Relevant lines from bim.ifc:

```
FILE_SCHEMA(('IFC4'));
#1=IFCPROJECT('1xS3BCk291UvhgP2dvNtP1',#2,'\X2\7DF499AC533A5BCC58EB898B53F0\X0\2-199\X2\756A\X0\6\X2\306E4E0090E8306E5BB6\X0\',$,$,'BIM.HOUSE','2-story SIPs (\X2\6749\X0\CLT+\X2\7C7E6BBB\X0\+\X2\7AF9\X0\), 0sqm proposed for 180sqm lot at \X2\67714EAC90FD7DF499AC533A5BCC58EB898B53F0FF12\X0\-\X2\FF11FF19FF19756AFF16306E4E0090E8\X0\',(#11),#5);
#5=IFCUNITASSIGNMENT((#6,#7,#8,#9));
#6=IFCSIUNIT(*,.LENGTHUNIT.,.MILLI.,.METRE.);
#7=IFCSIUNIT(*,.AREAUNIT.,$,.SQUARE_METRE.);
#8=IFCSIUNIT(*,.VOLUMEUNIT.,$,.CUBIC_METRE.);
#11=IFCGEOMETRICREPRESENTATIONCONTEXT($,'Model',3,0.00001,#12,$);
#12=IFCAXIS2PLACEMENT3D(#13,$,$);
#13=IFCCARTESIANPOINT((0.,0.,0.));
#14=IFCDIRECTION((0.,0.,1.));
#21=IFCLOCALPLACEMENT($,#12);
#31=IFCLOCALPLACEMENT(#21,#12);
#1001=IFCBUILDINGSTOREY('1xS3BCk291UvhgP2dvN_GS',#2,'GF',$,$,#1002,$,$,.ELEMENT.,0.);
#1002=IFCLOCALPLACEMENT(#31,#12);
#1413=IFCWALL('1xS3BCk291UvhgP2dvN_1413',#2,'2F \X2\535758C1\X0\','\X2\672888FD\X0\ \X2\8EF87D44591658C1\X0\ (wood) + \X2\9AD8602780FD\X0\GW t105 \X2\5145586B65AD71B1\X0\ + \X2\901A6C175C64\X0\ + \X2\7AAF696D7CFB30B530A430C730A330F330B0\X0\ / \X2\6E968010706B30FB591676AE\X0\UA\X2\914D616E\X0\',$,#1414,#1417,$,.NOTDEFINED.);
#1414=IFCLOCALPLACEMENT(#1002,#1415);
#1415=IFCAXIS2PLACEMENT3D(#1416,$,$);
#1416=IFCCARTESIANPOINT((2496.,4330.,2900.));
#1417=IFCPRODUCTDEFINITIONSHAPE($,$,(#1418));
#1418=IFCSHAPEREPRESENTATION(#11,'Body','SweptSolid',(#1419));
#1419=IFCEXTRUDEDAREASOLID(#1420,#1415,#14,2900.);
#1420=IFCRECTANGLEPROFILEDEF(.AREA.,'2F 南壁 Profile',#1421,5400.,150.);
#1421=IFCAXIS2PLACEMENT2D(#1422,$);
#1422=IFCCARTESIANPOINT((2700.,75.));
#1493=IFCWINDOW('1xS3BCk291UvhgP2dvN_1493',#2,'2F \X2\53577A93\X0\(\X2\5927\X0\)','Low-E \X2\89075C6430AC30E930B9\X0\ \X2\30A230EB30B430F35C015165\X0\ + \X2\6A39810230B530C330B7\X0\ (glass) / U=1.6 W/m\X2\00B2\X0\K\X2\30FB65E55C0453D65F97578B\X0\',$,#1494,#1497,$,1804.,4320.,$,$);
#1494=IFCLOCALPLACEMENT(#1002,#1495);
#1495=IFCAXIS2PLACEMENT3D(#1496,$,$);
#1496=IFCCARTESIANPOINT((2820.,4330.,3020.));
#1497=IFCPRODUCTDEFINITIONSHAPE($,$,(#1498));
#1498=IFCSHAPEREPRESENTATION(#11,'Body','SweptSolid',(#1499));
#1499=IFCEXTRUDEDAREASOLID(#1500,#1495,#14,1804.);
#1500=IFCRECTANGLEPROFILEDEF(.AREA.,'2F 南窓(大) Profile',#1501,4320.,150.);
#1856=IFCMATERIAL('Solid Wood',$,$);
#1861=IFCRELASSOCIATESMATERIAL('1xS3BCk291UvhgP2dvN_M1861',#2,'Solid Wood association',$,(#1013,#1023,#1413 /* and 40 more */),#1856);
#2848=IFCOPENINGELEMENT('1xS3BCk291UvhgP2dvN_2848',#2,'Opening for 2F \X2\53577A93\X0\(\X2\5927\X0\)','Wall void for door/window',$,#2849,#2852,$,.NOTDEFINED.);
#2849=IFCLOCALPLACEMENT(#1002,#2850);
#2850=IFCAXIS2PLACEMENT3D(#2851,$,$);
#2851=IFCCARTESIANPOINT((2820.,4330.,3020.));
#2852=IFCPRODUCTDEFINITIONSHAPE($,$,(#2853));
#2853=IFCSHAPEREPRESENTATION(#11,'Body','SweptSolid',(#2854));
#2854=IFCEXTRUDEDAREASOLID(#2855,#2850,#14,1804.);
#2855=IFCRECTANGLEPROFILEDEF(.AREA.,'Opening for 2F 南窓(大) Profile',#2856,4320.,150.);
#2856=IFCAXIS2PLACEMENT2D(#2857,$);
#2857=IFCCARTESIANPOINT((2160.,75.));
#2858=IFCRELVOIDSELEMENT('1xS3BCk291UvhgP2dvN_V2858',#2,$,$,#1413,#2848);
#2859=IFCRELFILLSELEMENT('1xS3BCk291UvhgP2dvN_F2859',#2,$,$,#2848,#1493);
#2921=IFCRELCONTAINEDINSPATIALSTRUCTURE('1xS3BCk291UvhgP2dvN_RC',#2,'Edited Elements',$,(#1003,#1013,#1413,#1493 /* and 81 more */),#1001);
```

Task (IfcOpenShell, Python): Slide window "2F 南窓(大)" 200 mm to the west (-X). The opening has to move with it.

```python
import ifcopenshell
import ifcopenshell.api.geometry
import ifcopenshell.util.placement

model = ifcopenshell.open("bim.ifc")

window = model.by_guid("1xS3BCk291UvhgP2dvN_1493")
opening = window.FillsVoids[0].RelatingOpeningElement
wall = opening.VoidsElements[0].RelatingBuildingElement

wall_matrix = ifcopenshell.util.placement.get_local_placement(wall.ObjectPlacement)
shift = wall_matrix[:3, 0] * -200.0
before = ifcopenshell.util.placement.get_local_placement(window.ObjectPlacement)[:3, 3].copy()

# The window is not placed relative to its opening, so move both.
for product in (opening, window):
    matrix = ifcopenshell.util.placement.get_local_placement(product.ObjectPlacement)
    matrix[:3, 3] += shift
    ifcopenshell.api.geometry.edit_object_placement(model, product=product, matrix=matrix, is_si=False)

after = ifcopenshell.util.placement.get_local_placement(window.ObjectPlacement)[:3, 3]
print("window moved by", (after - before).round(3) + 0.0)

model.write("bim_rev.ifc")
```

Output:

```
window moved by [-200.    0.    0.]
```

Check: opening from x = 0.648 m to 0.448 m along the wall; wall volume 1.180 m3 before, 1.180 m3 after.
